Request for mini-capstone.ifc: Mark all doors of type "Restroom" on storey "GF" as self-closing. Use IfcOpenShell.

First a look at what the model holds.

```python
import ifcopenshell
import ifcopenshell.util.element

model = ifcopenshell.open("mini-capstone.ifc")
print(model.schema)
storey = next(s for s in model.by_type("IfcBuildingStorey") if s.Name == "GF")
doors = [e for e in ifcopenshell.util.element.get_decomposition(storey) if e.is_a("IfcDoor")]
seen = {}
for e in doors:
    element_type = ifcopenshell.util.element.get_type(e)
    key = (element_type.Name if element_type != e and element_type else None, ifcopenshell.util.element.get_pset(e, "Pset_DoorCommon", "SelfClosing"))
    seen[key] = seen.get(key, 0) + 1
for (name, value), count in sorted(seen.items(), key=str):
    print(count, "x", name, "|", value)
```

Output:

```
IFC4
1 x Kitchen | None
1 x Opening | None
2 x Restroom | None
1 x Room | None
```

```python
import ifcopenshell
import ifcopenshell.api.pset
import ifcopenshell.util.element

model = ifcopenshell.open("mini-capstone.ifc")

storey = next(s for s in model.by_type("IfcBuildingStorey") if s.Name == "GF")
doors = [e for e in ifcopenshell.util.element.get_decomposition(storey) if e.is_a("IfcDoor")]

count = 0
for e in doors:
    element_type = ifcopenshell.util.element.get_type(e)
    if element_type in (None, e) or element_type.Name != "Restroom":
        continue
    # add_pset returns the element's existing set when there is one.
    pset = ifcopenshell.api.pset.add_pset(model, product=e, name="Pset_DoorCommon")
    ifcopenshell.api.pset.edit_pset(model, pset=pset, properties={"SelfClosing": True})
    count += 1

print(count, "doors updated")

model.write("mini-capstone_v2.ifc")
```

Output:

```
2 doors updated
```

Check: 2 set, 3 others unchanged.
